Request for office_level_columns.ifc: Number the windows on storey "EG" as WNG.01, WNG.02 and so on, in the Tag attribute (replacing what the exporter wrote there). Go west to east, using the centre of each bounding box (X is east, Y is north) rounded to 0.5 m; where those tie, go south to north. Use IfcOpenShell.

First a look at what the model holds.

```python
import ifcopenshell
import ifcopenshell.util.element
import ifcopenshell.util.placement

model = ifcopenshell.open("office_level_columns.ifc")
print(model.schema)
storey = next(s for s in model.by_type("IfcBuildingStorey") if s.Name == "EG")
windows = [e for e in ifcopenshell.util.element.get_decomposition(storey) if e.is_a("IfcWindow")]
for e in sorted(windows, key=lambda e: e.id()):
    origin = ifcopenshell.util.placement.get_local_placement(e.ObjectPlacement)[:3, 3]
    print(e.id(), e.Tag, e.Name, origin.round(2) + 0.0, sep=" | ")
```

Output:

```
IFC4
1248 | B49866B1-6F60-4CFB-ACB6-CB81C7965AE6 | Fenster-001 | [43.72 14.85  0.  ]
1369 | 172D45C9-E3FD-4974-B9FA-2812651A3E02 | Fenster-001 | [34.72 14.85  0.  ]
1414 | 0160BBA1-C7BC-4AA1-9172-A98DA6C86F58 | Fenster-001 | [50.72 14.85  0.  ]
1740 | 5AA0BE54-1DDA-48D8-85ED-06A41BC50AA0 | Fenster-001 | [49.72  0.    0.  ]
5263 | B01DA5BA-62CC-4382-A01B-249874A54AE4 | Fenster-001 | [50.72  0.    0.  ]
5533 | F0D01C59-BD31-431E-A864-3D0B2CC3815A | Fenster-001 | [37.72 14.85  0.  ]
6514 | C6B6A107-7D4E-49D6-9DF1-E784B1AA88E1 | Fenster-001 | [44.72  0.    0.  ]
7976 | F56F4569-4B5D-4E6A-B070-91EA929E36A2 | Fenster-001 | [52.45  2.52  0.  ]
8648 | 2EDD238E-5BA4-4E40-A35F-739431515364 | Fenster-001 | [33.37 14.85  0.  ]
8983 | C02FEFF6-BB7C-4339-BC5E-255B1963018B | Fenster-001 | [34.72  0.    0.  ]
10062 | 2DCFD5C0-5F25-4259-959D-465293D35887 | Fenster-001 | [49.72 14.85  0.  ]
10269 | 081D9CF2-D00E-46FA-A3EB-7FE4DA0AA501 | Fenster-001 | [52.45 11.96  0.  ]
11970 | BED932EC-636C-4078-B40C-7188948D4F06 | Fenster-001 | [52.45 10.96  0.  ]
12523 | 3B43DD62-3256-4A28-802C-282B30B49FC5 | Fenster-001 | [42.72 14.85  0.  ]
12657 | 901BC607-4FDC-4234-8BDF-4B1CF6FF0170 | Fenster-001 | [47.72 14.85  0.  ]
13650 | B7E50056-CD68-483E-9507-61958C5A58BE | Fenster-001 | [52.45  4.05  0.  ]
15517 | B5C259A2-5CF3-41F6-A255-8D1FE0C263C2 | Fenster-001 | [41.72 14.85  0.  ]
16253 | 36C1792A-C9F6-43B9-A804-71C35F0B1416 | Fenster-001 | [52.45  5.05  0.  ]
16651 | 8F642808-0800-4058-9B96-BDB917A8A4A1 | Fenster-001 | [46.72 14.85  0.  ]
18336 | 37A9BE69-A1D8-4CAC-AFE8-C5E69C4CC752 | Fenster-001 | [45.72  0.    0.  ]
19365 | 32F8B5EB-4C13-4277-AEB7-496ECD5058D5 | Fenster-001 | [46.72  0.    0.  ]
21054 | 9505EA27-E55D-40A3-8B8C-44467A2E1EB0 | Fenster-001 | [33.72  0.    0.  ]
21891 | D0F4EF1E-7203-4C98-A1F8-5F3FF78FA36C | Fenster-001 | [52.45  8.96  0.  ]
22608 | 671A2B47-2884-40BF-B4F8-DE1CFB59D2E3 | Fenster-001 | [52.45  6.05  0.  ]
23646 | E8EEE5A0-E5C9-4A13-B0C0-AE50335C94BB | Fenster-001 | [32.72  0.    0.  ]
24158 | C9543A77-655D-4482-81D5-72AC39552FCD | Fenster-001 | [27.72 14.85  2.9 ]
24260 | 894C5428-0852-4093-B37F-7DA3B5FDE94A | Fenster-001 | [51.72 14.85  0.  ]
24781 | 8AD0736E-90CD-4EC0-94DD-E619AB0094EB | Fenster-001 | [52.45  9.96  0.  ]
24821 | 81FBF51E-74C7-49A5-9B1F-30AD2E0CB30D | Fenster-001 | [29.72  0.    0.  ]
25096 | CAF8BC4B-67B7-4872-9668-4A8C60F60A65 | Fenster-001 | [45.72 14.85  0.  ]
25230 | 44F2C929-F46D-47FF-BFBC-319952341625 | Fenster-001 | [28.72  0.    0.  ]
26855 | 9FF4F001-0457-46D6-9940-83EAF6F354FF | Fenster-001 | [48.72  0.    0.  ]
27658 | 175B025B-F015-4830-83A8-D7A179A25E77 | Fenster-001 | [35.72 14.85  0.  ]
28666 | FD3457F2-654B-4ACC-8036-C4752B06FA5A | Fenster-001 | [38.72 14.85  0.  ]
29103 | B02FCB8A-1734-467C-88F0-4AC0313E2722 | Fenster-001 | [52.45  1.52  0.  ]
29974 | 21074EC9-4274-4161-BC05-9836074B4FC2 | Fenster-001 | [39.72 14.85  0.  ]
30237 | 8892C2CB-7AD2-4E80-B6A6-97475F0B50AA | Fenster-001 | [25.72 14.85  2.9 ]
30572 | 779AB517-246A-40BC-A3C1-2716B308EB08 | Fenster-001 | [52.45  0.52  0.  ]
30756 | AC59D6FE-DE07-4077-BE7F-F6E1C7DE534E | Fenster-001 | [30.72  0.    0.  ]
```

```python
import ifcopenshell
import ifcopenshell.geom
import ifcopenshell.util.element
import ifcopenshell.util.shape

model = ifcopenshell.open("office_level_columns.ifc")
settings = ifcopenshell.geom.settings()
settings.set("use-world-coords", True)


def centre(element):
    shape = ifcopenshell.geom.create_shape(settings, element)
    return ifcopenshell.util.shape.get_bbox_centroid(shape.geometry)


storey = next(s for s in model.by_type("IfcBuildingStorey") if s.Name == "EG")
windows = [e for e in ifcopenshell.util.element.get_decomposition(storey) if e.is_a("IfcWindow")]

# Insertion points can sit at a corner or the storey origin, so sort by the geometry (in metres).
centres = {e: centre(e) for e in windows}
windows.sort(key=lambda e: (round(centres[e][0] / 0.5), centres[e][1]))

for i, e in enumerate(windows, start=1):
    number = f"WNG.{i:02d}"
    e.Tag = number
    print(e.id(), number)

model.write("office_level_columns_v2.ifc")
```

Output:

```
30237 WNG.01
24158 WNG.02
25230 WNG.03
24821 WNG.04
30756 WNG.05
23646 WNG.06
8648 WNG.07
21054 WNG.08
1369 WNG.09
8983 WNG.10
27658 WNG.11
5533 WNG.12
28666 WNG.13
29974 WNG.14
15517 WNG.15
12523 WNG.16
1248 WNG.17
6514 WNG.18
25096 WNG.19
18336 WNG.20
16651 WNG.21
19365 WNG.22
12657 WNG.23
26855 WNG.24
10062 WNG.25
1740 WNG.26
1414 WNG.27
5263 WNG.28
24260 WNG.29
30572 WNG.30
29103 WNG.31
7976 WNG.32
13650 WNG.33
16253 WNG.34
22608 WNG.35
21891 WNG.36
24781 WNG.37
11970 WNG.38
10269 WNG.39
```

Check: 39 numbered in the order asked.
